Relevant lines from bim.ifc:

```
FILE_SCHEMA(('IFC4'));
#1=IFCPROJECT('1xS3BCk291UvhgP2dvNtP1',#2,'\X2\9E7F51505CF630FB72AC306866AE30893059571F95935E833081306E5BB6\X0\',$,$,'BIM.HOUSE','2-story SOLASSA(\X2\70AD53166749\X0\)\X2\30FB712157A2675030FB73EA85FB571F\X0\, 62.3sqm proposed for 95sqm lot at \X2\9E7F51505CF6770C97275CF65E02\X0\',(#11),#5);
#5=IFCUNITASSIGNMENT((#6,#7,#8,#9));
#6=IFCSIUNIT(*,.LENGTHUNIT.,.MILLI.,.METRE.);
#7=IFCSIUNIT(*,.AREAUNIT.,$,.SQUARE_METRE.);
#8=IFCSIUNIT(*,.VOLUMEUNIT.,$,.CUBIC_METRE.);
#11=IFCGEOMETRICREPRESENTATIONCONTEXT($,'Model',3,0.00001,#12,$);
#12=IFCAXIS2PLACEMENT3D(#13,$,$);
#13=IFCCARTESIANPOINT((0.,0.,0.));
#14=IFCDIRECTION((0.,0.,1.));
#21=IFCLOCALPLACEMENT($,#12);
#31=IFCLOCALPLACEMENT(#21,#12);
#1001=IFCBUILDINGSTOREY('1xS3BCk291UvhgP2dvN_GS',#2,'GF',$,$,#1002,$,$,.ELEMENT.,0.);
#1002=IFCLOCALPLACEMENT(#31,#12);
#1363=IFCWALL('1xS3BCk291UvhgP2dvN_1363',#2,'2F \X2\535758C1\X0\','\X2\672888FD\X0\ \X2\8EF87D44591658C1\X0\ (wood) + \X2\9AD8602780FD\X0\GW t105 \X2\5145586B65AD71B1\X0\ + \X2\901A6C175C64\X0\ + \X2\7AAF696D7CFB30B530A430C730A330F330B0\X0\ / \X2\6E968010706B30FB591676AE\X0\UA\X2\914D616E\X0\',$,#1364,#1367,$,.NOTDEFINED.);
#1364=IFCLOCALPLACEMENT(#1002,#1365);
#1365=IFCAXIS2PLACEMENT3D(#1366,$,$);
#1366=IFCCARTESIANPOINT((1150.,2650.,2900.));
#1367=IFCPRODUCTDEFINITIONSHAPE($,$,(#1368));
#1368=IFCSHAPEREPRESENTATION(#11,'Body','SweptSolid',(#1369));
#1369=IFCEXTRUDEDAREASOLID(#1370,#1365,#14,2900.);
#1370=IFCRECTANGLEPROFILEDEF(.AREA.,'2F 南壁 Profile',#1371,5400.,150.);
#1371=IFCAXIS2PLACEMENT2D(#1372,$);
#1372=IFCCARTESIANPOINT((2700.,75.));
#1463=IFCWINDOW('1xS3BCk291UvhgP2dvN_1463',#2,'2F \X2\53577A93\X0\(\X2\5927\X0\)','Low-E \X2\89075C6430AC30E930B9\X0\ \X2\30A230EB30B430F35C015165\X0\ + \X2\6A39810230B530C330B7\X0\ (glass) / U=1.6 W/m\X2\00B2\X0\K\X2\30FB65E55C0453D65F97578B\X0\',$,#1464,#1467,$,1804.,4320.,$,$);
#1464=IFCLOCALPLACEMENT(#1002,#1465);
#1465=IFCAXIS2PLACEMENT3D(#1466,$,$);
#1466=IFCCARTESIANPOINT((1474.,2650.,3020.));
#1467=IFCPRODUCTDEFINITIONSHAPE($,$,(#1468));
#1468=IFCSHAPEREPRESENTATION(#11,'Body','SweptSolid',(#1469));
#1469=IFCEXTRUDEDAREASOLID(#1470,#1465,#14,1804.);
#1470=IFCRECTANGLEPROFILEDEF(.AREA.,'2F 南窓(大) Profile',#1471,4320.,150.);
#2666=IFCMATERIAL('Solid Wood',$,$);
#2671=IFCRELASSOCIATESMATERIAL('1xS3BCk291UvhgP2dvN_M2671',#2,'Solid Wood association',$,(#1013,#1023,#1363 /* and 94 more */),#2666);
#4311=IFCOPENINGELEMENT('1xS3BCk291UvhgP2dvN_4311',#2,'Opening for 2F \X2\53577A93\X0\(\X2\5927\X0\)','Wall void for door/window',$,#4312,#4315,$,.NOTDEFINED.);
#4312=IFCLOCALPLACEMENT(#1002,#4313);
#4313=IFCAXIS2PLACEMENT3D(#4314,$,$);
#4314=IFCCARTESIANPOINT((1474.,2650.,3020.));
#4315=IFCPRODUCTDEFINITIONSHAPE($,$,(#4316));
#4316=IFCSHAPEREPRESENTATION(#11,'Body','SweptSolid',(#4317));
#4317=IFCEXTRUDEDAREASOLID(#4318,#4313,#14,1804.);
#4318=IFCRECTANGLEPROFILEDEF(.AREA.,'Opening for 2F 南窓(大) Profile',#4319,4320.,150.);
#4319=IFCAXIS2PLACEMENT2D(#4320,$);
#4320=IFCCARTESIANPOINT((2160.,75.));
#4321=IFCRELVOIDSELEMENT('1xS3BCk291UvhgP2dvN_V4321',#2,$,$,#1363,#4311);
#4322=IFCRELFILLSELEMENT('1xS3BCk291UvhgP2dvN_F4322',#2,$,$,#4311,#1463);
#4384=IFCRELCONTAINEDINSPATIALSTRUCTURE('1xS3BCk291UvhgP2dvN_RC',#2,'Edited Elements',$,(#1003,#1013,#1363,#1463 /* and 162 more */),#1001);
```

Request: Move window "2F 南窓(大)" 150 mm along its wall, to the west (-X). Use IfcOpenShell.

```python
import ifcopenshell
import ifcopenshell.api.geometry
import ifcopenshell.util.placement

model = ifcopenshell.open("bim.ifc")

window = model.by_guid("1xS3BCk291UvhgP2dvN_1463")
opening = window.FillsVoids[0].RelatingOpeningElement
wall = opening.VoidsElements[0].RelatingBuildingElement

wall_matrix = ifcopenshell.util.placement.get_local_placement(wall.ObjectPlacement)
shift = wall_matrix[:3, 0] * -150.0
before = ifcopenshell.util.placement.get_local_placement(window.ObjectPlacement)[:3, 3].copy()

# The window is not placed relative to its opening, so move both.
for product in (opening, window):
    matrix = ifcopenshell.util.placement.get_local_placement(product.ObjectPlacement)
    matrix[:3, 3] += shift
    ifcopenshell.api.geometry.edit_object_placement(model, product=product, matrix=matrix, is_si=False)

after = ifcopenshell.util.placement.get_local_placement(window.ObjectPlacement)[:3, 3]
print("window moved by", (after - before).round(3) + 0.0)

model.write("bim_edited.ifc")
```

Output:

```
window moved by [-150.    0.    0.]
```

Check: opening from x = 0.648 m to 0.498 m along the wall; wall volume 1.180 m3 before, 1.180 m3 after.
